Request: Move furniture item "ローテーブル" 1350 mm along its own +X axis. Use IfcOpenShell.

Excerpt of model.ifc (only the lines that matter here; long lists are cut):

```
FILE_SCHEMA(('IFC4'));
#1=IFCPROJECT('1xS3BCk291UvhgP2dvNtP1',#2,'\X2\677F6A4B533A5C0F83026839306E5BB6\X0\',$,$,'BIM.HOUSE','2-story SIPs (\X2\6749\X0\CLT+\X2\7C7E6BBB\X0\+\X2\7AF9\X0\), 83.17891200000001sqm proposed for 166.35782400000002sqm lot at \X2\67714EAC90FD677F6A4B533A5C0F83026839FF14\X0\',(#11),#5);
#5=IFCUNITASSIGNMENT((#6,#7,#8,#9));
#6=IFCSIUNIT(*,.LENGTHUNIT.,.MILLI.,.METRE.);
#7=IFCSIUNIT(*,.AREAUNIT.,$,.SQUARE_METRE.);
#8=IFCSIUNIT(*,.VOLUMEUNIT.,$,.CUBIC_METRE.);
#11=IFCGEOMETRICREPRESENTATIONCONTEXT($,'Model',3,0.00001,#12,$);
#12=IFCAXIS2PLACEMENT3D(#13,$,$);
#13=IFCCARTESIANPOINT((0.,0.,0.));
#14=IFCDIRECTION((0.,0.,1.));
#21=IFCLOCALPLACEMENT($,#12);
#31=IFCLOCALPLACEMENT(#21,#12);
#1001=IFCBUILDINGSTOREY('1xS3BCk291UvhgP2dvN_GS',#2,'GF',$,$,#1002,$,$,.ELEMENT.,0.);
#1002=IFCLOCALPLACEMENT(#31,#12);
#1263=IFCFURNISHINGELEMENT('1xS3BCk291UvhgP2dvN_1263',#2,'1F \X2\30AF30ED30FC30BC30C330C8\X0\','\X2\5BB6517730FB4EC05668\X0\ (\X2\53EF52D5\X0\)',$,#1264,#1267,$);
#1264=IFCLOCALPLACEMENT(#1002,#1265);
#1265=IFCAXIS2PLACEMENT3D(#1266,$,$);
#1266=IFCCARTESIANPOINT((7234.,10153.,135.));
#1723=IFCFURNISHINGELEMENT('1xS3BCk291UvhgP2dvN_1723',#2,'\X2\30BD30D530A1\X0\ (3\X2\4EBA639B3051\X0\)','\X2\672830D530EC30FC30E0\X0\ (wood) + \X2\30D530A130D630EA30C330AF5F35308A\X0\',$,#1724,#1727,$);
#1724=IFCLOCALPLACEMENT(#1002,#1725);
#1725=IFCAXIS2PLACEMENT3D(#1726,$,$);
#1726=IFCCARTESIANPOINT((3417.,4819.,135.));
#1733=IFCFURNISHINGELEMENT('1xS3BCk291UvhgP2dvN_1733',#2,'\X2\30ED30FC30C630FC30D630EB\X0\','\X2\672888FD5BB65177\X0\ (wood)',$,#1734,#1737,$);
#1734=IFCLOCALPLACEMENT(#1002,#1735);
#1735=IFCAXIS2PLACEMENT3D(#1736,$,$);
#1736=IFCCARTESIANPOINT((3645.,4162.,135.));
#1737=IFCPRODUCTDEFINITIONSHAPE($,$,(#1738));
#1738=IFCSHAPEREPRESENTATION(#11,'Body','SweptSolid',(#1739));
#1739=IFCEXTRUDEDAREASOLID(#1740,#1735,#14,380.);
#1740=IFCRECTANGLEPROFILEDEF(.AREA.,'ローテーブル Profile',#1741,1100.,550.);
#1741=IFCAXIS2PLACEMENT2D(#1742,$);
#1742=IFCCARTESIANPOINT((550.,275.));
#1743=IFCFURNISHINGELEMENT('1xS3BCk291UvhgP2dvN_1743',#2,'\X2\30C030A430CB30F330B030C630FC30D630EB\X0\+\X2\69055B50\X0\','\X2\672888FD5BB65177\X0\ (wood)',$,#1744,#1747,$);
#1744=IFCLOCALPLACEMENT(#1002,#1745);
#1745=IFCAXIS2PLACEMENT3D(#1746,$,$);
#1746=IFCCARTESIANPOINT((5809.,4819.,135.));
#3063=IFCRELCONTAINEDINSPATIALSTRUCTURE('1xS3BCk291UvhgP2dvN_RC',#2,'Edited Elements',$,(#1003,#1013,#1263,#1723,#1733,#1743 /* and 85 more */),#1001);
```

```python
import ifcopenshell
import ifcopenshell.api.geometry
import ifcopenshell.util.placement
import ifcopenshell.util.unit

model = ifcopenshell.open("model.ifc")
unit_scale = ifcopenshell.util.unit.calculate_unit_scale(model)

item = model.by_guid("1xS3BCk291UvhgP2dvN_1733")
matrix = ifcopenshell.util.placement.get_local_placement(item.ObjectPlacement)
matrix[:3, 3] += matrix[:3, 0] * 1.35 / unit_scale
ifcopenshell.api.geometry.edit_object_placement(model, product=item, matrix=matrix, is_si=False)

print(ifcopenshell.util.placement.get_local_placement(item.ObjectPlacement).round(3) + 0.0)

model.write("model_edited.ifc")
```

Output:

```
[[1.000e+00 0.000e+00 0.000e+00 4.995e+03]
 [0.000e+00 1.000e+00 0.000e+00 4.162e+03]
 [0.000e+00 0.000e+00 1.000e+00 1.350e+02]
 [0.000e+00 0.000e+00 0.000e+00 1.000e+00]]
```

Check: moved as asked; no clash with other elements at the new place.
